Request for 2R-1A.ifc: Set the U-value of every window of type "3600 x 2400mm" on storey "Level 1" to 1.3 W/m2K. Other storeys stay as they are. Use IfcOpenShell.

First a look at what the model holds.

```python
import ifcopenshell
import ifcopenshell.util.element

model = ifcopenshell.open("2R-1A.ifc")
print(model.schema)
storey = next(s for s in model.by_type("IfcBuildingStorey") if s.Name == "Level 1")
windows = [e for e in ifcopenshell.util.element.get_decomposition(storey) if e.is_a("IfcWindow")]
seen = {}
for e in windows:
    element_type = ifcopenshell.util.element.get_type(e)
    key = (element_type.Name if element_type != e and element_type else None, ifcopenshell.util.element.get_pset(e, "Pset_WindowCommon", "ThermalTransmittance"))
    seen[key] = seen.get(key, 0) + 1
for (name, value), count in sorted(seen.items(), key=str):
    print(count, "x", name, "|", value)
```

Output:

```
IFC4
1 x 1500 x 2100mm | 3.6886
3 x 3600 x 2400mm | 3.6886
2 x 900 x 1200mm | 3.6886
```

```python
import ifcopenshell
import ifcopenshell.api.pset
import ifcopenshell.util.element

model = ifcopenshell.open("2R-1A.ifc")

storey = next(s for s in model.by_type("IfcBuildingStorey") if s.Name == "Level 1")
windows = [e for e in ifcopenshell.util.element.get_decomposition(storey) if e.is_a("IfcWindow")]

count = 0
for e in windows:
    element_type = ifcopenshell.util.element.get_type(e)
    if element_type in (None, e) or element_type.Name != "3600 x 2400mm":
        continue
    # add_pset returns the element's existing set when there is one.
    pset = ifcopenshell.api.pset.add_pset(model, product=e, name="Pset_WindowCommon")
    ifcopenshell.api.pset.edit_pset(model, pset=pset, properties={"ThermalTransmittance": 1.3})
    count += 1

print(count, "windows updated")

model.write("2R-1A_rev.ifc")
```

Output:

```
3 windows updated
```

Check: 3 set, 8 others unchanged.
